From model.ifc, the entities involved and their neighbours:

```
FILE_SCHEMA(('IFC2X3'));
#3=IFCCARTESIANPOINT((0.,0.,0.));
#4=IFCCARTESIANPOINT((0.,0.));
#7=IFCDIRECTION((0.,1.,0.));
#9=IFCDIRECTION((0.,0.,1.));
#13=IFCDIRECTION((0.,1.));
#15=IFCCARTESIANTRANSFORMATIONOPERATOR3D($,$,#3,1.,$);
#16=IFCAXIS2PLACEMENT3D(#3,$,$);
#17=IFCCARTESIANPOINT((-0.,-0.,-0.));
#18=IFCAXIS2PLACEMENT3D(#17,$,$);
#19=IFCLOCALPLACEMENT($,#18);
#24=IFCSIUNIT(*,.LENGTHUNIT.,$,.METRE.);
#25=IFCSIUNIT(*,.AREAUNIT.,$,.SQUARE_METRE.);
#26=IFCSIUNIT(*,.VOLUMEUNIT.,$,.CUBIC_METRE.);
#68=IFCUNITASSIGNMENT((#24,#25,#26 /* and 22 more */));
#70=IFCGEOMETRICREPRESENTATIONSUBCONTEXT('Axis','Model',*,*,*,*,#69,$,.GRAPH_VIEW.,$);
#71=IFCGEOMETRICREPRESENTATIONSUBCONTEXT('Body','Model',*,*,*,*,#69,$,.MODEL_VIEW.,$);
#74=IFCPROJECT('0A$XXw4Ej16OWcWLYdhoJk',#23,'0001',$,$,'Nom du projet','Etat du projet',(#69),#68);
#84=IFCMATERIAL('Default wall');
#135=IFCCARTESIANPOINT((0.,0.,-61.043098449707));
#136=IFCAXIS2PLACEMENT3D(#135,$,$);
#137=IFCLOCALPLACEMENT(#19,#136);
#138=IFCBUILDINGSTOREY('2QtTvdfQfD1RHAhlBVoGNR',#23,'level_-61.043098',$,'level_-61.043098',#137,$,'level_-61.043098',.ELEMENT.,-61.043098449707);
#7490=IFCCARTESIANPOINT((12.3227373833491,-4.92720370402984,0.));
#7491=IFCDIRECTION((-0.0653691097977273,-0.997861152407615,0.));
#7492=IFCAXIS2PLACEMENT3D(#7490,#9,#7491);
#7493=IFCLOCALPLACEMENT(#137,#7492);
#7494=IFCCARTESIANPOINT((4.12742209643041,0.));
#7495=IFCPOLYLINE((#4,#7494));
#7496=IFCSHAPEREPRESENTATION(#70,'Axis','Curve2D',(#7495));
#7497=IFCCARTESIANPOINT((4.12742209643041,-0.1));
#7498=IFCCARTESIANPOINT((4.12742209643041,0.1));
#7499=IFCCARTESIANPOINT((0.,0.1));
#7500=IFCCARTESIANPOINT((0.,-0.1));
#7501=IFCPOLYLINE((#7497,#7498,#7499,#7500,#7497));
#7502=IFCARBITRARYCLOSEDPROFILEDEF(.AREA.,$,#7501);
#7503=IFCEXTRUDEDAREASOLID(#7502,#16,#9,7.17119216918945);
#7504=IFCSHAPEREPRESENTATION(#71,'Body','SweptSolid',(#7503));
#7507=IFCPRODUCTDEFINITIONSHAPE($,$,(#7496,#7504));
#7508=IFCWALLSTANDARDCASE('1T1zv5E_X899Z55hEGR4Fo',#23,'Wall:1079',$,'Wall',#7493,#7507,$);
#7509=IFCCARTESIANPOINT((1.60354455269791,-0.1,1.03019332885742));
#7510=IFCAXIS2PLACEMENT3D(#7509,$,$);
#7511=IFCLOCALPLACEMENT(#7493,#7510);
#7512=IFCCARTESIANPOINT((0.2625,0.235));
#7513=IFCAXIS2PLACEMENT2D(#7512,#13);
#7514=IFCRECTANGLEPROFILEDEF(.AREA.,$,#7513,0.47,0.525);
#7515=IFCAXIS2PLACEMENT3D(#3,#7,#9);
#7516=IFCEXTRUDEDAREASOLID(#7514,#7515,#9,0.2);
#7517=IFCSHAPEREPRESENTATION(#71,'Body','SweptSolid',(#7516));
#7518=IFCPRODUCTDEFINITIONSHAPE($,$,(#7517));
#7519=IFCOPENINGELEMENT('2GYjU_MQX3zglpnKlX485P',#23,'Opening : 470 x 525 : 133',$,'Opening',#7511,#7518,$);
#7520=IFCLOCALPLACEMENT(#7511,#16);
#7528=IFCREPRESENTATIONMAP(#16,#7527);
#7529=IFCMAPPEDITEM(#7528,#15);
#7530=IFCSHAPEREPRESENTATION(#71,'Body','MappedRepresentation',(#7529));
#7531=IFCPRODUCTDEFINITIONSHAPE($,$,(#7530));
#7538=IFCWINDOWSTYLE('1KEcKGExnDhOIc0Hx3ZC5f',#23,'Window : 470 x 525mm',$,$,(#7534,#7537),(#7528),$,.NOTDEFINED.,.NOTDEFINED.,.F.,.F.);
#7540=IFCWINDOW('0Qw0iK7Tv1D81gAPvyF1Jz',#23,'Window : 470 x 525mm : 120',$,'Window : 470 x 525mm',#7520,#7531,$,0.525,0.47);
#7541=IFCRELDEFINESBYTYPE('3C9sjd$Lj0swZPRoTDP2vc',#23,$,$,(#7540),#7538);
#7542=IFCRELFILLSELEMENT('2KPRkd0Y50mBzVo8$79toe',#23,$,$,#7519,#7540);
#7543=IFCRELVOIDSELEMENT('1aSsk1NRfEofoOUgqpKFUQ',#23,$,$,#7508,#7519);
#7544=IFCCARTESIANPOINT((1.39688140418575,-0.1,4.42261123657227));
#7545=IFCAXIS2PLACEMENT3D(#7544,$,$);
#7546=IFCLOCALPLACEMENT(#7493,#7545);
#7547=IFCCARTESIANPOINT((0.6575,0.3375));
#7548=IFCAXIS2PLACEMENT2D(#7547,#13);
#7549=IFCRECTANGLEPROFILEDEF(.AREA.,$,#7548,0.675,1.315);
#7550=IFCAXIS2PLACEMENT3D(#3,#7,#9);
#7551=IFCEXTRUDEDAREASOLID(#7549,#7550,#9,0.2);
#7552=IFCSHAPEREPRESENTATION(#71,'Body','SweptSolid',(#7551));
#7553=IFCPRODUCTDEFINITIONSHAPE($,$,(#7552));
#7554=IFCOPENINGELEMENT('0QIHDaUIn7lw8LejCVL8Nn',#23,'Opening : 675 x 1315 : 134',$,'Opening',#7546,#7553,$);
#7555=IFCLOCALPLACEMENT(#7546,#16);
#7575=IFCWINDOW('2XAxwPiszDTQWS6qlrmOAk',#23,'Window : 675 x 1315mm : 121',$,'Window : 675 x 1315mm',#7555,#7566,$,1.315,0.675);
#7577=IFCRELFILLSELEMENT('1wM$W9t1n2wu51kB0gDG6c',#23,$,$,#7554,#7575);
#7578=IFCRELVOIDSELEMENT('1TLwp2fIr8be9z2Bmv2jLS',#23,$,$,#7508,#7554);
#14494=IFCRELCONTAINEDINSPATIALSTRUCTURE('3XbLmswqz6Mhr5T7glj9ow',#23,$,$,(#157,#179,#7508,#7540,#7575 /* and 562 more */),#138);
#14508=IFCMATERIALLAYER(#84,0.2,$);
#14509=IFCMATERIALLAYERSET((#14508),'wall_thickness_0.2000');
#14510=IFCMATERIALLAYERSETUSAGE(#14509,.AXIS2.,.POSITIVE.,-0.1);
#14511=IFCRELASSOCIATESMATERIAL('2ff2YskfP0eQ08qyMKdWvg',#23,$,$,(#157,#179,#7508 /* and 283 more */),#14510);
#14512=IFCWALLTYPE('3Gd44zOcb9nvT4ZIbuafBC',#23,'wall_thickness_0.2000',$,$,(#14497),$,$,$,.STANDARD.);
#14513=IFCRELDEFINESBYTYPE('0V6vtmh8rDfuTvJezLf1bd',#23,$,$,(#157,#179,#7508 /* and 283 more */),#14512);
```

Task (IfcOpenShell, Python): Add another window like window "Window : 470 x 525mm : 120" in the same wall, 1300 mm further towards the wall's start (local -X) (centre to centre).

```python
import ifcopenshell
import ifcopenshell.api.feature
import ifcopenshell.api.geometry
import ifcopenshell.api.root
import ifcopenshell.geom
import ifcopenshell.util.element
import ifcopenshell.util.placement
import ifcopenshell.util.shape
import ifcopenshell.util.unit

model = ifcopenshell.open("model.ifc")
unit_scale = ifcopenshell.util.unit.calculate_unit_scale(model)
settings = ifcopenshell.geom.settings()


def volume(element):
    """Net volume in cubic metres, openings subtracted."""
    shape = ifcopenshell.geom.create_shape(settings, element)
    return ifcopenshell.util.shape.get_volume(shape.geometry)


window = model.by_id(7540)
opening = window.FillsVoids[0].RelatingOpeningElement
wall = opening.VoidsElements[0].RelatingBuildingElement
before = volume(wall)
shift = ifcopenshell.util.placement.get_local_placement(wall.ObjectPlacement)[:3, 0] * -1.3 / unit_scale

# copy_class copies the void relationship, type, container and properties, but no geometry.
new_opening = ifcopenshell.api.root.copy_class(model, product=opening)
new_opening.Representation = ifcopenshell.util.element.copy_deep(
    model, opening.Representation, exclude=["IfcGeometricRepresentationContext", "IfcRepresentationMap"]
)
new_opening.Name = "Opening : 470 x 525"
new_window = ifcopenshell.api.root.copy_class(model, product=window)
new_window.Representation = ifcopenshell.util.element.copy_deep(
    model, window.Representation, exclude=["IfcGeometricRepresentationContext", "IfcRepresentationMap"]
)
new_window.Name = "Window : 470 x 525mm"
fills = ifcopenshell.api.feature.add_filling(model, opening=new_opening, element=new_window)
fills.OwnerHistory = new_window.OwnerHistory  # required in IFC2X3

for old, new in ((opening, new_opening), (window, new_window)):
    matrix = ifcopenshell.util.placement.get_local_placement(old.ObjectPlacement)
    matrix[:3, 3] += shift
    ifcopenshell.api.geometry.edit_object_placement(model, product=new, matrix=matrix, is_si=False)

after = volume(wall)

print(f"wall volume {before:.3f} -> {after:.3f} m3")

model.write("model_edited.ifc")
```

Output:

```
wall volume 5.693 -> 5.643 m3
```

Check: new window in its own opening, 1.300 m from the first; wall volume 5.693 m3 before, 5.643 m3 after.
